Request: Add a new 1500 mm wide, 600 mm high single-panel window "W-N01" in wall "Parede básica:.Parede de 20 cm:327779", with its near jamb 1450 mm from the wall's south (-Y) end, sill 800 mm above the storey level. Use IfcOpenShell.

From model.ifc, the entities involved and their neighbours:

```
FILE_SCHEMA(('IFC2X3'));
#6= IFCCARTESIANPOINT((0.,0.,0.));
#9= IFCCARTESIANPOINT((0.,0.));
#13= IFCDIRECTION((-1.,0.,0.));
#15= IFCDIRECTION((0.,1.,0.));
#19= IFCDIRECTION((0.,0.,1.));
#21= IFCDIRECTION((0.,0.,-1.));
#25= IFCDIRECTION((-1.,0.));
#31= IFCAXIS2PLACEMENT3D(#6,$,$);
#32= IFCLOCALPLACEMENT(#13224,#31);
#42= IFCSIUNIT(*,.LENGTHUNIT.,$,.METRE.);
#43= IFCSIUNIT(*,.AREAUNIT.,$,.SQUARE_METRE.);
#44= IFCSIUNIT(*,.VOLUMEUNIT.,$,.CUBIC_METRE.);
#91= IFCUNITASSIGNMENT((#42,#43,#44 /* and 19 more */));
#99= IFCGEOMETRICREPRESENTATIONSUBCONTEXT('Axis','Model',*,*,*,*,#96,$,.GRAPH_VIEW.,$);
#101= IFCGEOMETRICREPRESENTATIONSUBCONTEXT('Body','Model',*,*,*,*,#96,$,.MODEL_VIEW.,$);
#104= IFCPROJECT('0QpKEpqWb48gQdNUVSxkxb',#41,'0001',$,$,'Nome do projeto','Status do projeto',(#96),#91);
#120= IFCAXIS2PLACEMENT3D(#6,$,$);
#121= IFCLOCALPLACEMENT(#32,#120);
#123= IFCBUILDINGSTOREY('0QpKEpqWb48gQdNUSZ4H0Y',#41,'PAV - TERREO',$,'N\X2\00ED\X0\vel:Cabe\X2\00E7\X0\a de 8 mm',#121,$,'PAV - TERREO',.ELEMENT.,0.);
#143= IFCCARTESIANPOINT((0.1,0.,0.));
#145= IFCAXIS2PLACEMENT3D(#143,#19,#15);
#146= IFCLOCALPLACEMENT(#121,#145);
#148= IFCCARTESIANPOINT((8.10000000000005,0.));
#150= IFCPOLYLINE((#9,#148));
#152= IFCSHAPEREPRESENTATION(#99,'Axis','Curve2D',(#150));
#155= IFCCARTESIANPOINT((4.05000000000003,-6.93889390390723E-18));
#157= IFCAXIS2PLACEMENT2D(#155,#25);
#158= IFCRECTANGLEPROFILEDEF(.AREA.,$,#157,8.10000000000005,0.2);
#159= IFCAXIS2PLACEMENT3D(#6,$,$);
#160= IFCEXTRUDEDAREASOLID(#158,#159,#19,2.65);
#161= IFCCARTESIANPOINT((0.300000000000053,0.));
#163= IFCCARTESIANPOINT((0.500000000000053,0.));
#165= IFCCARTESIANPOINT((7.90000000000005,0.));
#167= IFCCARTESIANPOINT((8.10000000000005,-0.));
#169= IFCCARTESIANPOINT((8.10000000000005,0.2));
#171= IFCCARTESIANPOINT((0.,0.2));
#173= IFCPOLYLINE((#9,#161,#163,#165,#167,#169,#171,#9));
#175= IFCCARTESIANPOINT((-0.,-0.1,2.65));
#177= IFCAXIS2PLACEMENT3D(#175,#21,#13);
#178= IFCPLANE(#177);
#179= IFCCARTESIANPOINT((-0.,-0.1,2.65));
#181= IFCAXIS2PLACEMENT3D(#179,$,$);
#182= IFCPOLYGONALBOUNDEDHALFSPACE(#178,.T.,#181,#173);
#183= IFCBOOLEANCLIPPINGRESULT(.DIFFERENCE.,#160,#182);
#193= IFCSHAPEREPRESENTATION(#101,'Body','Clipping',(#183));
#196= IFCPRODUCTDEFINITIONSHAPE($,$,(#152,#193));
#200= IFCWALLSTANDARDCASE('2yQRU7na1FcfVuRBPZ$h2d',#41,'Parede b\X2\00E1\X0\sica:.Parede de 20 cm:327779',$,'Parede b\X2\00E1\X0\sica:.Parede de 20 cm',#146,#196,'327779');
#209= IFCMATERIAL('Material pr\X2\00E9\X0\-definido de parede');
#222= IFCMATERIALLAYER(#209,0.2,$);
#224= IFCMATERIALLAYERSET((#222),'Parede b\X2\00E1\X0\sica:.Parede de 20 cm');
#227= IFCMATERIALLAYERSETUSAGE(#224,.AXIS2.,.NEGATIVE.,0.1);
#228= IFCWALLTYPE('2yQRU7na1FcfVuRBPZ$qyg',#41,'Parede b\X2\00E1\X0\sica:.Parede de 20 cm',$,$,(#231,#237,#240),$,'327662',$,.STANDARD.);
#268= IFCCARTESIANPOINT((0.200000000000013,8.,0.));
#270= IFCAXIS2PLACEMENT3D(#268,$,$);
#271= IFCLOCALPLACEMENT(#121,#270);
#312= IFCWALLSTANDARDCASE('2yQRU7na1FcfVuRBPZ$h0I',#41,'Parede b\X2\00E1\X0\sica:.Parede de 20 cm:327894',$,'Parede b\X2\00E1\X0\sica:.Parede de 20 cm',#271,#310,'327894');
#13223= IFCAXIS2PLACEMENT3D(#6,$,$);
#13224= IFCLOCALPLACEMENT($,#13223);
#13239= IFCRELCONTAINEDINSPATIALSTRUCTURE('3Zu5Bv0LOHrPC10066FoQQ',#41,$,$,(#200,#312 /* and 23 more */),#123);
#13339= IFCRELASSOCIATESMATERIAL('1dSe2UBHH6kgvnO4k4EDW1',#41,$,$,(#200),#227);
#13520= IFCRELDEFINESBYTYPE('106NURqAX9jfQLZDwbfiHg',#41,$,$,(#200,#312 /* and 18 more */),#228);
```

```python
import numpy as np
import ifcopenshell
import ifcopenshell.api.feature
import ifcopenshell.api.geometry
import ifcopenshell.api.root
import ifcopenshell.api.spatial
import ifcopenshell.api.type
import ifcopenshell.geom
import ifcopenshell.util.element
import ifcopenshell.util.placement
import ifcopenshell.util.representation
import ifcopenshell.util.shape
import ifcopenshell.util.unit

model = ifcopenshell.open("model.ifc")
unit_scale = ifcopenshell.util.unit.calculate_unit_scale(model)
settings = ifcopenshell.geom.settings()


def volume(element):
    """Net volume in cubic metres, openings subtracted."""
    shape = ifcopenshell.geom.create_shape(settings, element)
    return ifcopenshell.util.shape.get_volume(shape.geometry)


wall = model.by_guid("2yQRU7na1FcfVuRBPZ$h2d")
storey = ifcopenshell.util.element.get_container(wall, ifc_class="IfcBuildingStorey")
context = ifcopenshell.util.representation.get_context(model, "Model", "Body", "MODEL_VIEW")
before = volume(wall)

width, height, from_end, sill = 1.5, 0.6, 1.45, 0.8  # metres

# The wall runs along its own X axis, and the end named is its -X end.
wall_shape = ifcopenshell.geom.create_shape(settings, wall)
x, y, z = ifcopenshell.util.shape.get_vertices(wall_shape.geometry).T
start = x.min() + from_end
face, thickness = float(y.min()), float(y.max() - y.min())
wall_matrix = ifcopenshell.util.placement.get_local_placement(wall.ObjectPlacement)
level = ifcopenshell.util.placement.get_local_placement(storey.ObjectPlacement)[2, 3]


def in_wall(x, y):
    """Placement at x, y metres in the wall's axes, at sill height."""
    matrix = wall_matrix.copy()
    matrix[:, 3] = wall_matrix @ np.array([x / unit_scale, y / unit_scale, 0.0, 1.0])
    matrix[2, 3] = level + sill / unit_scale
    return matrix


# Opening: a box that overshoots both wall faces by 50 mm.
opening = ifcopenshell.api.root.create_entity(model, ifc_class="IfcOpeningElement")
box = ifcopenshell.api.geometry.add_wall_representation(
    model, context=context, length=width, height=height, thickness=thickness + 0.1
)
ifcopenshell.api.geometry.assign_representation(model, product=opening, representation=box)
ifcopenshell.api.geometry.edit_object_placement(model, product=opening, matrix=in_wall(start, face - 0.05), is_si=False)
ifcopenshell.api.feature.add_feature(model, feature=opening, element=wall)

window = ifcopenshell.api.root.create_entity(model, ifc_class="IfcWindow", name="W-N01")
window.OverallWidth, window.OverallHeight = width / unit_scale, height / unit_scale
body = ifcopenshell.api.geometry.add_window_representation(
    model,
    context=context,
    overall_width=window.OverallWidth,
    overall_height=window.OverallHeight,
    partition_type="SINGLE_PANEL",
)
ifcopenshell.api.geometry.assign_representation(model, product=window, representation=body)
ifcopenshell.api.spatial.assign_container(model, products=[window], relating_structure=storey)
fills = ifcopenshell.api.feature.add_filling(model, opening=opening, element=window)
fills.OwnerHistory = window.OwnerHistory  # required in IFC2X3

# IFC2X3 keeps the operation on the window style.
style = ifcopenshell.api.root.create_entity(model, ifc_class="IfcWindowStyle", name="W-N01")
style.OperationType, style.ConstructionType = "SINGLE_PANEL", "NOTDEFINED"
style.ParameterTakesPrecedence = style.Sizeable = False
ifcopenshell.api.type.assign_type(model, related_objects=[window], relating_type=style)

# Centre the window in the wall's thickness.
ifcopenshell.api.geometry.edit_object_placement(model, product=window, matrix=in_wall(start, face), is_si=False)
window_shape = ifcopenshell.geom.create_shape(settings, window)
depth = ifcopenshell.util.shape.get_vertices(window_shape.geometry)[:, 1]
offset = face + thickness / 2 - (depth.min() + depth.max()) / 2
ifcopenshell.api.geometry.edit_object_placement(model, product=window, matrix=in_wall(start, offset), is_si=False)

after = volume(wall)

print(f"wall volume {before:.3f} -> {after:.3f} m3")

model.write("model_rev.ifc")
```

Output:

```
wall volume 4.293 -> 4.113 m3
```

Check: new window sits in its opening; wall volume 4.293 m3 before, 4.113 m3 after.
